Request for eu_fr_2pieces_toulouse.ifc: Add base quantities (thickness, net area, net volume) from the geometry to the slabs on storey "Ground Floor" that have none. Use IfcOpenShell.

First a look at what the model holds.

```python
import ifcopenshell
import ifcopenshell.util.element
import ifcopenshell.util.unit

model = ifcopenshell.open("eu_fr_2pieces_toulouse.ifc")
print(model.schema)
for unit_type in ("LENGTHUNIT", "AREAUNIT", "VOLUMEUNIT"):
    print(unit_type, ifcopenshell.util.unit.calculate_unit_scale(model, unit_type))
storey = next(s for s in model.by_type("IfcBuildingStorey") if s.Name == "Ground Floor")
slabs = [e for e in ifcopenshell.util.element.get_decomposition(storey) if e.is_a("IfcSlab")]
for e in sorted(slabs, key=lambda e: e.id()):
    print(e.id(), e.is_a(), e.Name, list(ifcopenshell.util.element.get_psets(e, qtos_only=True)), sep=" | ")
```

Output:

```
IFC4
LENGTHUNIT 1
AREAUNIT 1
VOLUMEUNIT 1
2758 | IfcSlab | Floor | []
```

```python
import ifcopenshell
import ifcopenshell.api.pset
import ifcopenshell.geom
import ifcopenshell.util.element
import ifcopenshell.util.shape
import ifcopenshell.util.unit

model = ifcopenshell.open("eu_fr_2pieces_toulouse.ifc")
unit_scale = ifcopenshell.util.unit.calculate_unit_scale(model)
area_scale = ifcopenshell.util.unit.calculate_unit_scale(model, "AREAUNIT")
volume_scale = ifcopenshell.util.unit.calculate_unit_scale(model, "VOLUMEUNIT")
settings = ifcopenshell.geom.settings()

storey = next(s for s in model.by_type("IfcBuildingStorey") if s.Name == "Ground Floor")
slabs = [e for e in ifcopenshell.util.element.get_decomposition(storey) if e.is_a("IfcSlab")]

for e in sorted(slabs, key=lambda e: e.id()):
    if ifcopenshell.util.element.get_psets(e, qtos_only=True, should_inherit=False):
        continue
    # Geometry comes back in metres, in the element's own axes.
    shape = ifcopenshell.geom.create_shape(settings, e)
    values = {
        "Width": ifcopenshell.util.shape.get_z(shape.geometry) / unit_scale,
        "NetArea": ifcopenshell.util.shape.get_footprint_area(shape.geometry) / area_scale,
        "NetVolume": ifcopenshell.util.shape.get_volume(shape.geometry) / volume_scale,
    }
    qto = ifcopenshell.api.pset.add_qto(model, product=e, name="Qto_SlabBaseQuantities")
    ifcopenshell.api.pset.edit_qto(model, qto=qto, properties=values)
    print(e.id(), {k: round(v, 3) for k, v in values.items()})

model.write("eu_fr_2pieces_toulouse_updated.ifc")
```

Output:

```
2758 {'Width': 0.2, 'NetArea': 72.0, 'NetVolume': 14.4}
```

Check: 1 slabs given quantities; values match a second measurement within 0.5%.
